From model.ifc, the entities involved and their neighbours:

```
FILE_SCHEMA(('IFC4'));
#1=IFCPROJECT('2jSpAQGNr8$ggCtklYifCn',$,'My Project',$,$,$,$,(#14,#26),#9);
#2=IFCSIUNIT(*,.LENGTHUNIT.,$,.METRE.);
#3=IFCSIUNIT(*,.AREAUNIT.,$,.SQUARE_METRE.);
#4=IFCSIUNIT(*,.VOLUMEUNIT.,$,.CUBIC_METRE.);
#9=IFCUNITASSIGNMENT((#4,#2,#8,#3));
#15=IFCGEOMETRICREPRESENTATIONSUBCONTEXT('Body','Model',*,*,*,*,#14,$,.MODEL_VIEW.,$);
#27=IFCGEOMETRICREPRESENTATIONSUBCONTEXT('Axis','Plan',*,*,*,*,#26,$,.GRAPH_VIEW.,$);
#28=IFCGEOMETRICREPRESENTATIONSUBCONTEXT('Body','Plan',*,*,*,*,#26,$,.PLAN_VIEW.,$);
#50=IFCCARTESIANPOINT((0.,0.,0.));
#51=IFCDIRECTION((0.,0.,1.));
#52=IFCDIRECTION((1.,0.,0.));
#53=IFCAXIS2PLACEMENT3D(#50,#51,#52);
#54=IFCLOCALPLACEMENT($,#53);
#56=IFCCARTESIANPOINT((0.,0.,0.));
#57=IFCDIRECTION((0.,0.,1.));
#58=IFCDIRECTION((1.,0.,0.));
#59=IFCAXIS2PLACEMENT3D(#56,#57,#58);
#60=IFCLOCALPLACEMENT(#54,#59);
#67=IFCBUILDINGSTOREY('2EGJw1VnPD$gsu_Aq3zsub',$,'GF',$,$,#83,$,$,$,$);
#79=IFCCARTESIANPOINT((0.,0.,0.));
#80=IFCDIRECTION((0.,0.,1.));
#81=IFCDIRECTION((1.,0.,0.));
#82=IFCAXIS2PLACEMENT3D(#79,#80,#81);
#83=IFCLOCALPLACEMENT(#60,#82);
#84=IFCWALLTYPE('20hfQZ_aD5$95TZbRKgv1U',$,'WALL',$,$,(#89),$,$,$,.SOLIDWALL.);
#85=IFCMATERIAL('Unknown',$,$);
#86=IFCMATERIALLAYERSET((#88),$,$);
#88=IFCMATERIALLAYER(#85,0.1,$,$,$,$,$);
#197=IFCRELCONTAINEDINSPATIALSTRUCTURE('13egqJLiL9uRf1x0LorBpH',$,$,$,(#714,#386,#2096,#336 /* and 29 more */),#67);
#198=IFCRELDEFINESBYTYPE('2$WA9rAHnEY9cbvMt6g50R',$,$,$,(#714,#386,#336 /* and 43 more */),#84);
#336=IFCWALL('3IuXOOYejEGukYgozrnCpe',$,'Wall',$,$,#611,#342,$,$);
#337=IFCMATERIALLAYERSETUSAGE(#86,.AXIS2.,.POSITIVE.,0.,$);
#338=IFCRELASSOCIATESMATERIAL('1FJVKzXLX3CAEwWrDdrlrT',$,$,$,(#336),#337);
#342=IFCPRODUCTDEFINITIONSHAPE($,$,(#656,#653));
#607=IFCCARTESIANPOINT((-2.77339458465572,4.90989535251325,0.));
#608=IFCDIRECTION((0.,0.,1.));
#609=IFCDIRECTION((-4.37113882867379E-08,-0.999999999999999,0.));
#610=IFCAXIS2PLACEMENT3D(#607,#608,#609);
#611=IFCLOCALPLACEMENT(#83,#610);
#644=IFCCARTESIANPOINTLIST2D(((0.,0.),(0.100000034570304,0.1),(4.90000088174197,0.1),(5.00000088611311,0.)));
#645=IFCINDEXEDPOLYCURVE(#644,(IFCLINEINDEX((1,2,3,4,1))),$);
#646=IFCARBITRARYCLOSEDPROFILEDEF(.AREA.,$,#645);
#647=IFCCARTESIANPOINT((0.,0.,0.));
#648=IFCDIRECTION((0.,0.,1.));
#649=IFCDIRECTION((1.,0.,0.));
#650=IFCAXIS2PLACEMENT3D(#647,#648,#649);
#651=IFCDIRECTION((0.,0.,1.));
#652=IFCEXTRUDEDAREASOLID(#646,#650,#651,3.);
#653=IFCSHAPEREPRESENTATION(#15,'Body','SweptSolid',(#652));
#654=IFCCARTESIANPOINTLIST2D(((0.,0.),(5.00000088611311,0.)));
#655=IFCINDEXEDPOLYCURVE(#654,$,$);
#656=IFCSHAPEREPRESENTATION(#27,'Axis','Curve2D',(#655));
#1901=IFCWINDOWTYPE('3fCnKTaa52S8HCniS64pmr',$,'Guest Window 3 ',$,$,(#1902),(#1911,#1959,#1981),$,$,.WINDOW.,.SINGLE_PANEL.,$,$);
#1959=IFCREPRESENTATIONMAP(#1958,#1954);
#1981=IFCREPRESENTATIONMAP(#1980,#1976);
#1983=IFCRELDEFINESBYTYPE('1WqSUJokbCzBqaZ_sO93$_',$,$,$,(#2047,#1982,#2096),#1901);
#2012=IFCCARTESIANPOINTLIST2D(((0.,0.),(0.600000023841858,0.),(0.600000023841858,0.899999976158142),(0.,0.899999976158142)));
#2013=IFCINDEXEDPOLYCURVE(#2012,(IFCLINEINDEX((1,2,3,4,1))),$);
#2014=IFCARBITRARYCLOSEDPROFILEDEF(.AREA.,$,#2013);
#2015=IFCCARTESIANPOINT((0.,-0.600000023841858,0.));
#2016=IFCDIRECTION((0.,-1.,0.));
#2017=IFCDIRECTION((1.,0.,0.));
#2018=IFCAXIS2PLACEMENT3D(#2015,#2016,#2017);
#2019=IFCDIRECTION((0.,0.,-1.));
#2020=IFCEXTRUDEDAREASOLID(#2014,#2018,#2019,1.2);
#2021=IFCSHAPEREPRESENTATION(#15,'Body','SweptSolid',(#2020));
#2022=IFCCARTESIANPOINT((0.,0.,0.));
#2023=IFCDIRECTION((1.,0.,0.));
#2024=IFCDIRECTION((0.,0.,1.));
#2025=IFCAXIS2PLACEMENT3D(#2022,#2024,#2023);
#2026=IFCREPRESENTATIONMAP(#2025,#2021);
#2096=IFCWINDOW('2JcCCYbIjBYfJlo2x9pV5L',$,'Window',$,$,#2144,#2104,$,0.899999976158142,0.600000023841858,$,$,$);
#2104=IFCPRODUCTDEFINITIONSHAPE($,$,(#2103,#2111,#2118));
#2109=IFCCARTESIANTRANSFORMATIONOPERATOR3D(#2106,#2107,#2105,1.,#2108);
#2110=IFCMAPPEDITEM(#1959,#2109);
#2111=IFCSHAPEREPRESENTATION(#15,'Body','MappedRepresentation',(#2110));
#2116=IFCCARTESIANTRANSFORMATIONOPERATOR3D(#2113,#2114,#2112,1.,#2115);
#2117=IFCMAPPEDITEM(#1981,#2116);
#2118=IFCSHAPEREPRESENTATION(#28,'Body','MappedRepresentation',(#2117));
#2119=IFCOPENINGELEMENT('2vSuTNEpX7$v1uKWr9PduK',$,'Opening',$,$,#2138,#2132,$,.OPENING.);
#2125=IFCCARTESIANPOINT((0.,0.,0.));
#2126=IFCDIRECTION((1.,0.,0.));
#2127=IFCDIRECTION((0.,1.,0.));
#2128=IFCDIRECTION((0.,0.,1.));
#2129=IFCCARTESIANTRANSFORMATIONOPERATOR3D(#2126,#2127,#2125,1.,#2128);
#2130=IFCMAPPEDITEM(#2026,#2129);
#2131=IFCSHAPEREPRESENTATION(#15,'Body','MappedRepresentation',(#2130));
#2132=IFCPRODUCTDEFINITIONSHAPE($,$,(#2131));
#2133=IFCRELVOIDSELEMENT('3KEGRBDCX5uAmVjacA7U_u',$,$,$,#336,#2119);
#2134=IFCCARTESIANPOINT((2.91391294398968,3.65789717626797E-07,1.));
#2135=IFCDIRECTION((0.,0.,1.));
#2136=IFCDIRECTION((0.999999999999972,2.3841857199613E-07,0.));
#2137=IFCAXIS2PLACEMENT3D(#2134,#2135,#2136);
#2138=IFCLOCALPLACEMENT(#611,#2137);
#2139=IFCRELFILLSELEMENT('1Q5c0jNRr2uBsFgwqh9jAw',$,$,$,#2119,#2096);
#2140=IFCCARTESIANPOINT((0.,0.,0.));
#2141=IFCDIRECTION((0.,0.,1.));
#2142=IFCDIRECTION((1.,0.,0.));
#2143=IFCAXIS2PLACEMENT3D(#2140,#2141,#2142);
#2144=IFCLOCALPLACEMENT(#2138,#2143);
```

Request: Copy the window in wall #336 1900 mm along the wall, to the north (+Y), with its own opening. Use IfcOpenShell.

```python
import ifcopenshell
import ifcopenshell.api.feature
import ifcopenshell.api.geometry
import ifcopenshell.api.root
import ifcopenshell.geom
import ifcopenshell.util.element
import ifcopenshell.util.placement
import ifcopenshell.util.shape

model = ifcopenshell.open("model.ifc")
settings = ifcopenshell.geom.settings()


def volume(element):
    """Net volume in cubic metres, openings subtracted."""
    shape = ifcopenshell.geom.create_shape(settings, element)
    return ifcopenshell.util.shape.get_volume(shape.geometry)


window = model.by_id(2096)
opening = window.FillsVoids[0].RelatingOpeningElement
wall = opening.VoidsElements[0].RelatingBuildingElement
before = volume(wall)
shift = ifcopenshell.util.placement.get_local_placement(wall.ObjectPlacement)[:3, 0] * -1.9

# copy_class copies the void relationship, type, container and properties, but no geometry.
new_opening = ifcopenshell.api.root.copy_class(model, product=opening)
new_opening.Representation = ifcopenshell.util.element.copy_deep(
    model, opening.Representation, exclude=["IfcGeometricRepresentationContext", "IfcRepresentationMap"]
)
new_window = ifcopenshell.api.root.copy_class(model, product=window)
new_window.Representation = ifcopenshell.util.element.copy_deep(
    model, window.Representation, exclude=["IfcGeometricRepresentationContext", "IfcRepresentationMap"]
)
ifcopenshell.api.feature.add_filling(model, opening=new_opening, element=new_window)

for old, new in ((opening, new_opening), (window, new_window)):
    matrix = ifcopenshell.util.placement.get_local_placement(old.ObjectPlacement)
    matrix[:3, 3] += shift
    ifcopenshell.api.geometry.edit_object_placement(model, product=new, matrix=matrix, is_si=False)

after = volume(wall)

print(f"wall volume {before:.3f} -> {after:.3f} m3")

model.write("model_edited.ifc")
```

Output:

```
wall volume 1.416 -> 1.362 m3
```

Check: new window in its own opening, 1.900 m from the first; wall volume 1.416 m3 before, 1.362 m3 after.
